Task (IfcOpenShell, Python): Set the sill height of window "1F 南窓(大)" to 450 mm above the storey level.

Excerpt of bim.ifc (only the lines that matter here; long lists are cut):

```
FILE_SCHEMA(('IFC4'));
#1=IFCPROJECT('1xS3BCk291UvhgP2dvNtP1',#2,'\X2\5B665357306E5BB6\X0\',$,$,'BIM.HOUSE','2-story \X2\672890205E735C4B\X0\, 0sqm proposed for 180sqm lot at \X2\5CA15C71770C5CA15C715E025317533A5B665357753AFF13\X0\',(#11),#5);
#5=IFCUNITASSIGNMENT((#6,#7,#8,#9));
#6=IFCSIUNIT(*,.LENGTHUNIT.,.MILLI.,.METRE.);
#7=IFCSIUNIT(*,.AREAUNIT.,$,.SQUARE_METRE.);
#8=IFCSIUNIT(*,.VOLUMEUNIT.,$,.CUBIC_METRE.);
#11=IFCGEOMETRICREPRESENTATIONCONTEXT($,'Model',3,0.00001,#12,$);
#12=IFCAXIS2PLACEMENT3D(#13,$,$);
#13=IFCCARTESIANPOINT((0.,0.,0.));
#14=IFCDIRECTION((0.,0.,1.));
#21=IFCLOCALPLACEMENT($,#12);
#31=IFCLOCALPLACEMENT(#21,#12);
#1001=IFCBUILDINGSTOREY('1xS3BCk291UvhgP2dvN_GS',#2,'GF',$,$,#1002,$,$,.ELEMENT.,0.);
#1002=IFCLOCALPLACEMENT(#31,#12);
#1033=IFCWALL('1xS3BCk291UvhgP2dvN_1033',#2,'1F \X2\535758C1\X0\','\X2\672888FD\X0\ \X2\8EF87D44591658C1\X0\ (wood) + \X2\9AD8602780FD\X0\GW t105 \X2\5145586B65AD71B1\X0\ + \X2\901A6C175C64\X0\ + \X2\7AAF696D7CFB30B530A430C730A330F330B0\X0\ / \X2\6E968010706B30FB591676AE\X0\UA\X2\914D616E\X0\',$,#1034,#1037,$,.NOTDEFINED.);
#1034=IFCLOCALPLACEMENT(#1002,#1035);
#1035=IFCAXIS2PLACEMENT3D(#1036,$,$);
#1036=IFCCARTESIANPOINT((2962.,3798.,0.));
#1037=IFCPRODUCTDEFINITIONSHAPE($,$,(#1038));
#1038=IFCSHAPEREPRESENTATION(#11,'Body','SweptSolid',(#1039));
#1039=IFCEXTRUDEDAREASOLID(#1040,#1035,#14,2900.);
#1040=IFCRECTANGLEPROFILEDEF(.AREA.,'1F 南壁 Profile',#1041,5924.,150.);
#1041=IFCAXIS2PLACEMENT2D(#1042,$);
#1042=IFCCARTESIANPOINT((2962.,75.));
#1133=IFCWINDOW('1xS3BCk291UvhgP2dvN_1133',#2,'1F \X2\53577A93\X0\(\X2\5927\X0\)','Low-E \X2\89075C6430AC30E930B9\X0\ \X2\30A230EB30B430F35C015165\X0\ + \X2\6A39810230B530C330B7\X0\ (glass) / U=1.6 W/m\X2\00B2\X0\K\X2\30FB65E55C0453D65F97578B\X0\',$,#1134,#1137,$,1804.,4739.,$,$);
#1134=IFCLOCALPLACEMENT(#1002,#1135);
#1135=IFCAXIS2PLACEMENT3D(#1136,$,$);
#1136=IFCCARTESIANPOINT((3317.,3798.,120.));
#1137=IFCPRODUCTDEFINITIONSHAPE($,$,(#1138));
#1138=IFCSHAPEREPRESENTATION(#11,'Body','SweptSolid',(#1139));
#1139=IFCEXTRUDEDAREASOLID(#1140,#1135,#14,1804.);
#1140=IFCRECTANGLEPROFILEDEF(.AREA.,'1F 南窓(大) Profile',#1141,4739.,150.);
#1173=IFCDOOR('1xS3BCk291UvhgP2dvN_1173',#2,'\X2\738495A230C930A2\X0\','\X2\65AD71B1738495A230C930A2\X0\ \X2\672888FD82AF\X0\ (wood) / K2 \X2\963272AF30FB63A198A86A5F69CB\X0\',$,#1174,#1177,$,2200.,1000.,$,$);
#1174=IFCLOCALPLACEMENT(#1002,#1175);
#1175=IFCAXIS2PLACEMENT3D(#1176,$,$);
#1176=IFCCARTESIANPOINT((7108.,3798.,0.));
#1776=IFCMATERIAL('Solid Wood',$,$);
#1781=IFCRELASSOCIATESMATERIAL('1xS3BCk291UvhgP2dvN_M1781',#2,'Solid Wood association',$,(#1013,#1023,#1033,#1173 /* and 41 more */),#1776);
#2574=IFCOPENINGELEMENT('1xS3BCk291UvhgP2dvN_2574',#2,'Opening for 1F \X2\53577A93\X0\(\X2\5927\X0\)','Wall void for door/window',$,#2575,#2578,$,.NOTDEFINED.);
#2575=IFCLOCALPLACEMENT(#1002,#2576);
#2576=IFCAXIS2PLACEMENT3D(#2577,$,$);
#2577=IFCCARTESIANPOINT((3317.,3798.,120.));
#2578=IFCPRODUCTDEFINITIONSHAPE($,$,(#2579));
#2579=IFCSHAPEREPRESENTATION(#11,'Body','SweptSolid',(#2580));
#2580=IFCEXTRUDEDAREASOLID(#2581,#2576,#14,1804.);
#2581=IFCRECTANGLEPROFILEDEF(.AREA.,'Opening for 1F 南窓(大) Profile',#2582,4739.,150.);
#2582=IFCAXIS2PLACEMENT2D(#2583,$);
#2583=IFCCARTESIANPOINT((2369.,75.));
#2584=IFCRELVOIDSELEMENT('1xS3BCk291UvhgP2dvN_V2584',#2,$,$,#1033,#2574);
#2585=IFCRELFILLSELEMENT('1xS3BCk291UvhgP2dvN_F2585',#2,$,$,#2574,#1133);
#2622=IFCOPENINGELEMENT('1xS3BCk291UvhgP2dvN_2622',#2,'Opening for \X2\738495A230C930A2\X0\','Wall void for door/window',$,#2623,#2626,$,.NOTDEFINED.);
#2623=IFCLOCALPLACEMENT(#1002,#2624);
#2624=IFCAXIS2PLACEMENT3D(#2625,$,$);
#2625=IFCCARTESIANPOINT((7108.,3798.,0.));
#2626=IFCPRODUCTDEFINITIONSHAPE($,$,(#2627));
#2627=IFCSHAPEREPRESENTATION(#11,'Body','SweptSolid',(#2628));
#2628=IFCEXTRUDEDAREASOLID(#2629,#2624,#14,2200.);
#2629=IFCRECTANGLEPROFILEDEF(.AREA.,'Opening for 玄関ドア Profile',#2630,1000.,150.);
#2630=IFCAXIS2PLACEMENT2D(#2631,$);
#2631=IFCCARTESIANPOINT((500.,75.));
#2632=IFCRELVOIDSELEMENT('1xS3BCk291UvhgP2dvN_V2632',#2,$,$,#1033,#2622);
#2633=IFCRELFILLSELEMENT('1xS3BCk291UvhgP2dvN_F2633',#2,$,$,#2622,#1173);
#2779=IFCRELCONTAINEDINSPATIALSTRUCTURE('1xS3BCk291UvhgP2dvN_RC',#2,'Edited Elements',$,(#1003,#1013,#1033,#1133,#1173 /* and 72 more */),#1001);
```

```python
import numpy as np
import ifcopenshell
import ifcopenshell.api.geometry
import ifcopenshell.geom
import ifcopenshell.util.element
import ifcopenshell.util.placement
import ifcopenshell.util.shape
import ifcopenshell.util.unit

model = ifcopenshell.open("bim.ifc")
unit_scale = ifcopenshell.util.unit.calculate_unit_scale(model)

window = model.by_guid("1xS3BCk291UvhgP2dvN_1133")
opening = window.FillsVoids[0].RelatingOpeningElement
storey = ifcopenshell.util.element.get_container(window, ifc_class="IfcBuildingStorey")
level = ifcopenshell.util.placement.get_local_placement(storey.ObjectPlacement)[2, 3]

# The opening's origin need not be at the sill, so measure its lowest point.
shape = ifcopenshell.geom.create_shape(ifcopenshell.geom.settings(), opening)
bottom = ifcopenshell.util.shape.get_shape_bottom_elevation(shape, shape.geometry) / unit_scale
dz = level + 450.0 - bottom

shift = np.array([0.0, 0.0, dz])
# The window is not placed relative to its opening, so move both.
for product in (opening, window):
    matrix = ifcopenshell.util.placement.get_local_placement(product.ObjectPlacement)
    matrix[:3, 3] += shift
    ifcopenshell.api.geometry.edit_object_placement(model, product=product, matrix=matrix, is_si=False)

print(f"moved by {dz * unit_scale:+.3f} m")

model.write("bim_v2.ifc")
```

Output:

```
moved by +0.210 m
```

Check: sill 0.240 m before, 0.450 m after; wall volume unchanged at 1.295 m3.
